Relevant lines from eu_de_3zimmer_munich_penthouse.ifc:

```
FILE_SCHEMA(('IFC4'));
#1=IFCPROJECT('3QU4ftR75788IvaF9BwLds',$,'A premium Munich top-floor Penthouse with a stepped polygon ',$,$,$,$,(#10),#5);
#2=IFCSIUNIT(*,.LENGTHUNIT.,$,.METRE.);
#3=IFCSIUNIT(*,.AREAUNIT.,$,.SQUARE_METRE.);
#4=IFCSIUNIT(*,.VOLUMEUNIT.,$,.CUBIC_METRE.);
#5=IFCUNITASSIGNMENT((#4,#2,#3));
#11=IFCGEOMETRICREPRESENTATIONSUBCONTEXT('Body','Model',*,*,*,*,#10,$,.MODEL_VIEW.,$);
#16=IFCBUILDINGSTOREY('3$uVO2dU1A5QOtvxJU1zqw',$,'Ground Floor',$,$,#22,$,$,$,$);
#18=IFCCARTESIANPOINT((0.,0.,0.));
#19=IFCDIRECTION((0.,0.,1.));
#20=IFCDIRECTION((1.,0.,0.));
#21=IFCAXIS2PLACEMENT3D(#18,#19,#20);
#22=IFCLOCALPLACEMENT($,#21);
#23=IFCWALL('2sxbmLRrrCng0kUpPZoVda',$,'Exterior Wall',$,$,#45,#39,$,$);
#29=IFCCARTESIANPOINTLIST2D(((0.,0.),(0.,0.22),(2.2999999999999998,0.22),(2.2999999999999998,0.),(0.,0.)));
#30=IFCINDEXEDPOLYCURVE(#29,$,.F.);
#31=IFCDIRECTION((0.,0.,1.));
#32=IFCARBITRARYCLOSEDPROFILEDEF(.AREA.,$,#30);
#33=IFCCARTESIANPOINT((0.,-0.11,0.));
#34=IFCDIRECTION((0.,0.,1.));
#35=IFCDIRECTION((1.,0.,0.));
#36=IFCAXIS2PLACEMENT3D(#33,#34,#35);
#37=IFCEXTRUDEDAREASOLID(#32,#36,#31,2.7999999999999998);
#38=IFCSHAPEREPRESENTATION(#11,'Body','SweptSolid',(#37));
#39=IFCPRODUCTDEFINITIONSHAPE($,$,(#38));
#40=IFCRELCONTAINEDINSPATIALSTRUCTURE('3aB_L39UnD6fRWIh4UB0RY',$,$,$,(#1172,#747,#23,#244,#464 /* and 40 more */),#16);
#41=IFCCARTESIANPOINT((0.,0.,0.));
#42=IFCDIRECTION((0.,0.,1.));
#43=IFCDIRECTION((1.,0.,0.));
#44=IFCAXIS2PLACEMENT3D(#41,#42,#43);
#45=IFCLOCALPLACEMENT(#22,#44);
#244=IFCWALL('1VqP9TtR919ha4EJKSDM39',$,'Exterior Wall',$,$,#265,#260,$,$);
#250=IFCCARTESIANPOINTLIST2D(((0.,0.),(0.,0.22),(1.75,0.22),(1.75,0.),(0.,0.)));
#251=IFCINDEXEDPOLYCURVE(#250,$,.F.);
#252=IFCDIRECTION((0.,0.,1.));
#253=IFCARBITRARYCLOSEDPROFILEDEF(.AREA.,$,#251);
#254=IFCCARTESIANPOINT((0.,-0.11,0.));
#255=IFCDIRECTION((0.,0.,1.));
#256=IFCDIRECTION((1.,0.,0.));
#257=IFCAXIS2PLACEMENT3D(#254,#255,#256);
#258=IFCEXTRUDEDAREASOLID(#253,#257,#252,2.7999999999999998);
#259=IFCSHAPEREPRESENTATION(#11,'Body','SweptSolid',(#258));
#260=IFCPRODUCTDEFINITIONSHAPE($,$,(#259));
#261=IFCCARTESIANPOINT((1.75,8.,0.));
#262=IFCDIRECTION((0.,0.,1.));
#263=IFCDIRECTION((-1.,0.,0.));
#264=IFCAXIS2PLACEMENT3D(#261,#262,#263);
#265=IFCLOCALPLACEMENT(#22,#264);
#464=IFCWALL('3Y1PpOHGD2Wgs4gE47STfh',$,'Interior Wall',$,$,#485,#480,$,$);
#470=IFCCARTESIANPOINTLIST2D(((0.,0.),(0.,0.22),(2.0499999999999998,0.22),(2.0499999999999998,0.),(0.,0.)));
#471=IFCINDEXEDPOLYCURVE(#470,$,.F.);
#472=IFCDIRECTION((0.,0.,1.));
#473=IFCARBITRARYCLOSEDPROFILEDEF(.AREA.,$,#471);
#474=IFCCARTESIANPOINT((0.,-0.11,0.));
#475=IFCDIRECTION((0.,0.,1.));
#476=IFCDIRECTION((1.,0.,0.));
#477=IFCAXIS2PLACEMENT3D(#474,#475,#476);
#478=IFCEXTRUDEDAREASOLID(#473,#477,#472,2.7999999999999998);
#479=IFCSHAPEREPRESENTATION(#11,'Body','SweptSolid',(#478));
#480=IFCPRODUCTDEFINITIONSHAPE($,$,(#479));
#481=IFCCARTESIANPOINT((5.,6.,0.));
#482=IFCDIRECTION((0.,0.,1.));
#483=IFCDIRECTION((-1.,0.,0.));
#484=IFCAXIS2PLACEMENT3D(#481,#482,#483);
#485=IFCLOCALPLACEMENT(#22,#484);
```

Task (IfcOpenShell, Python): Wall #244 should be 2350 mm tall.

```python
import ifcopenshell
import ifcopenshell.geom
import ifcopenshell.util.representation
import ifcopenshell.util.shape
import ifcopenshell.util.unit

model = ifcopenshell.open("eu_de_3zimmer_munich_penthouse.ifc")
unit_scale = ifcopenshell.util.unit.calculate_unit_scale(model)
settings = ifcopenshell.geom.settings()


def volume(element):
    """Net volume in cubic metres, openings subtracted."""
    shape = ifcopenshell.geom.create_shape(settings, element)
    return ifcopenshell.util.shape.get_volume(shape.geometry)


wall = model.by_guid("1VqP9TtR919ha4EJKSDM39")
before = volume(wall)

body = ifcopenshell.util.representation.get_representation(wall, "Model", "Body")
solid = body.Items[0]
old_height = solid.Depth
solid.Depth = 2.35 / unit_scale
after = volume(wall)

print(f"height {old_height:g} -> {solid.Depth:g}, volume {before:.3f} -> {after:.3f} m3")

model.write("eu_de_3zimmer_munich_penthouse_rev.ifc")
```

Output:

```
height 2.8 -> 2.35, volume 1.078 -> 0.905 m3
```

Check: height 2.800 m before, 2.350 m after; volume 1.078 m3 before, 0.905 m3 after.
